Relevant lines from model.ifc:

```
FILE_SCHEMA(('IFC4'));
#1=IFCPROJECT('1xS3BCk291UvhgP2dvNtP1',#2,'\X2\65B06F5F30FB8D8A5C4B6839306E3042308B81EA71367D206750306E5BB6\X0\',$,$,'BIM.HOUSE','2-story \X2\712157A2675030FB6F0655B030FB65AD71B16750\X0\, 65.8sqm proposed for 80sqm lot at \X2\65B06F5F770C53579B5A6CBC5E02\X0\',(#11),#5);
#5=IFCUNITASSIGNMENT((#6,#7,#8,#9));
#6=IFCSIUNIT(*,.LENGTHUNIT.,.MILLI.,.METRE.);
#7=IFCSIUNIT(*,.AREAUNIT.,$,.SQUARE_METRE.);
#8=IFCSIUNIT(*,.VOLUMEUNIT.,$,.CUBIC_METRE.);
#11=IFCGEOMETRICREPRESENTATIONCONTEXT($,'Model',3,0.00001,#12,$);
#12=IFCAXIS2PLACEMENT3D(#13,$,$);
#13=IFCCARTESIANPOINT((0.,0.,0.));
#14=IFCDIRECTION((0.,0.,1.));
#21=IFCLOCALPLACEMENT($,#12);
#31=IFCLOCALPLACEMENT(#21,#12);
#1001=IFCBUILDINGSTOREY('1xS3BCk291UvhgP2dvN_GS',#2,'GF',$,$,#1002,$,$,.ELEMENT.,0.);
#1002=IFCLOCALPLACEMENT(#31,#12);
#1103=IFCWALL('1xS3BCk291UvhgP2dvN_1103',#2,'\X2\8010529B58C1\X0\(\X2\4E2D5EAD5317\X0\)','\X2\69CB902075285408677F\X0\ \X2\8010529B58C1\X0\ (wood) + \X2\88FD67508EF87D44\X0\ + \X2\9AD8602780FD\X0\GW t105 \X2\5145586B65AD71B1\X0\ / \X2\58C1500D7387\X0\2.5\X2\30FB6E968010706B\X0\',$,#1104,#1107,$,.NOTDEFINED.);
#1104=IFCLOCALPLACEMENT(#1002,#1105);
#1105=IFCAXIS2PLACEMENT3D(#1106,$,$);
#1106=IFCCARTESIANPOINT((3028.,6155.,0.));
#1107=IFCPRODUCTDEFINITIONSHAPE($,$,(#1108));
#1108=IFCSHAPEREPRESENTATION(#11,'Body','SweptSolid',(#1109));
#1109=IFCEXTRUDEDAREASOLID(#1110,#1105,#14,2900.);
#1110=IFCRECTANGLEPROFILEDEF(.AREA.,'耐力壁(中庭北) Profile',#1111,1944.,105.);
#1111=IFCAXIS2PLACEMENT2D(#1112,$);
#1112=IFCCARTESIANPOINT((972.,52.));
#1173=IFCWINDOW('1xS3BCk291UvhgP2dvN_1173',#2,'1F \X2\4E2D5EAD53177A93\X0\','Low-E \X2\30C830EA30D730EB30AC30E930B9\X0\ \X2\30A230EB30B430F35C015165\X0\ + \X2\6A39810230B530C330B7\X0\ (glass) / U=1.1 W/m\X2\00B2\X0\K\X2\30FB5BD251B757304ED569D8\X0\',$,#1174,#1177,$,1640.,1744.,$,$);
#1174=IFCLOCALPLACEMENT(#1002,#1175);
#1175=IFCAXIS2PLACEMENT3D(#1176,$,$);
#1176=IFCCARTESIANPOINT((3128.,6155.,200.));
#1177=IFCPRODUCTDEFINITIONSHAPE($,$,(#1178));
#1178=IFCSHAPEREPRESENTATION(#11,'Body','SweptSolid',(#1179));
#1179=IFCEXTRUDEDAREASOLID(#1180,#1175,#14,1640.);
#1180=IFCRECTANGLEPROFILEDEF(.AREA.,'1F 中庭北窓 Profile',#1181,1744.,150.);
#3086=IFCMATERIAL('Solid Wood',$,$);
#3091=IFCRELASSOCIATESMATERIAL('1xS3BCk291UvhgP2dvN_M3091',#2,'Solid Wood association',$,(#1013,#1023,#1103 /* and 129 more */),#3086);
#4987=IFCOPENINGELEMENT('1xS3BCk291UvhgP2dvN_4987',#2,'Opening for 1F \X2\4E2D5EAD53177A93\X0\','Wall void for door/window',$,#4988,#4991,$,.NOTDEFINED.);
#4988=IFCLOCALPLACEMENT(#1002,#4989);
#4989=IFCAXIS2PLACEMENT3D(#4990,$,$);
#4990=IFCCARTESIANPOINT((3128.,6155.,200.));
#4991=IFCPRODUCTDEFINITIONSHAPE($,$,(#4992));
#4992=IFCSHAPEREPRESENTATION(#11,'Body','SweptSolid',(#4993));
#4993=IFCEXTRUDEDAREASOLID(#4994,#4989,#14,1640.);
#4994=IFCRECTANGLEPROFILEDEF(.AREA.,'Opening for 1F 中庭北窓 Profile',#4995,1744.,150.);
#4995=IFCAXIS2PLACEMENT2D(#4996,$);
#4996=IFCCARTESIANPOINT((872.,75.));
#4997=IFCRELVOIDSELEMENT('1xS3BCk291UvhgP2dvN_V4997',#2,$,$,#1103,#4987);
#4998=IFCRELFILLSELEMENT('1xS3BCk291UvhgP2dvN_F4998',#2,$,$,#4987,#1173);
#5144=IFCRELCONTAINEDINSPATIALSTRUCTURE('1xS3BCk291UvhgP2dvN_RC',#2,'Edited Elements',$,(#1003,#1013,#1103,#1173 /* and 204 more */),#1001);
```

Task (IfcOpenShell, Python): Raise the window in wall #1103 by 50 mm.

```python
import numpy as np
import ifcopenshell
import ifcopenshell.api.geometry
import ifcopenshell.util.placement
import ifcopenshell.util.unit

model = ifcopenshell.open("model.ifc")
unit_scale = ifcopenshell.util.unit.calculate_unit_scale(model)

window = model.by_guid("1xS3BCk291UvhgP2dvN_1173")
opening = window.FillsVoids[0].RelatingOpeningElement
dz = 0.05 / unit_scale

shift = np.array([0.0, 0.0, dz])
# The window is not placed relative to its opening, so move both.
for product in (opening, window):
    matrix = ifcopenshell.util.placement.get_local_placement(product.ObjectPlacement)
    matrix[:3, 3] += shift
    ifcopenshell.api.geometry.edit_object_placement(model, product=product, matrix=matrix, is_si=False)

print(f"moved by {dz * unit_scale:+.3f} m")

model.write("model_updated.ifc")
```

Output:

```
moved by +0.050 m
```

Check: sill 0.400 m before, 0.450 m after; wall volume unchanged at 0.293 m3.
